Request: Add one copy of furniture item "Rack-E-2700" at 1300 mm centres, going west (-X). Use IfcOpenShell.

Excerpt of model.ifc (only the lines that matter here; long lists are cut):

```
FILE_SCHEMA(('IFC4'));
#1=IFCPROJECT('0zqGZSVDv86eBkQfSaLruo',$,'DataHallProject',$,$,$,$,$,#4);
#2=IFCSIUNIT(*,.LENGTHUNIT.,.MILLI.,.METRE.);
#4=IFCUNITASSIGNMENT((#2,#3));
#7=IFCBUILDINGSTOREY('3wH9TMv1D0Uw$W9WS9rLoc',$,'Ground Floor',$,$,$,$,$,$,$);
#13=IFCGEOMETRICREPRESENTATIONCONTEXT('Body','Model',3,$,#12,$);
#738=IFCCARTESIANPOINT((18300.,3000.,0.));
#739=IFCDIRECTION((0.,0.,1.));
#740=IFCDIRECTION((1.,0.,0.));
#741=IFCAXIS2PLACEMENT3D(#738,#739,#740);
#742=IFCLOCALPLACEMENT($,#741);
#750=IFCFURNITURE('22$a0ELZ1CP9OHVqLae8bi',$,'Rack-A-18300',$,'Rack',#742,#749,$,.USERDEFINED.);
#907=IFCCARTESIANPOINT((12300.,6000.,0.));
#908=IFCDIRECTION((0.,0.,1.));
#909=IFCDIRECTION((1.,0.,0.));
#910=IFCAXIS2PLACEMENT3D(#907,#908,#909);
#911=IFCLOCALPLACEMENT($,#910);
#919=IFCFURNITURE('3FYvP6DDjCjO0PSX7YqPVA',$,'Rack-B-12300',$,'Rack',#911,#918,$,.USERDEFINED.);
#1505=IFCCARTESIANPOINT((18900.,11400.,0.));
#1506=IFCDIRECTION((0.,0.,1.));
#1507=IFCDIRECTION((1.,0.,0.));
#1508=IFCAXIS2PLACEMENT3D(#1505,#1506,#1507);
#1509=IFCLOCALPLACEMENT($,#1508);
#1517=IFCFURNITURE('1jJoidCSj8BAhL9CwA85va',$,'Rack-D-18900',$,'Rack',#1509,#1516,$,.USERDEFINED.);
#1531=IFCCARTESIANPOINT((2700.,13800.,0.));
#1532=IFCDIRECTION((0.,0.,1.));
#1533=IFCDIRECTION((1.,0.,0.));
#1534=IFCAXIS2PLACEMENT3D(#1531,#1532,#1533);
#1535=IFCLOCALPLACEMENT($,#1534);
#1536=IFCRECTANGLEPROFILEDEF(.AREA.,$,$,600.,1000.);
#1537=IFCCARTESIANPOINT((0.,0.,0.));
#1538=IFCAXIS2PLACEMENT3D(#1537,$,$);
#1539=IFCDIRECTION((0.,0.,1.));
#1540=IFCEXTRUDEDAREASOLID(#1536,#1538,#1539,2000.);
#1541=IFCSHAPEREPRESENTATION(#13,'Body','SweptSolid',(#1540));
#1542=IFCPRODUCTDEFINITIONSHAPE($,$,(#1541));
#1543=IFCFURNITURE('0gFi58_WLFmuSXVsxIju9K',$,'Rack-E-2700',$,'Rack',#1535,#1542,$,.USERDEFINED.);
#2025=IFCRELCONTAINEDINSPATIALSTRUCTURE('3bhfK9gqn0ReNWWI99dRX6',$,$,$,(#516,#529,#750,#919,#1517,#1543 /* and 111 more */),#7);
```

```python
import numpy as np
import ifcopenshell
import ifcopenshell.api.geometry
import ifcopenshell.api.root
import ifcopenshell.util.element
import ifcopenshell.util.placement

model = ifcopenshell.open("model.ifc")

source = model.by_guid("0gFi58_WLFmuSXVsxIju9K")
base = ifcopenshell.util.placement.get_local_placement(source.ObjectPlacement)
step = np.array([-1.0, 0.0, 0.0]) * 1300.0

for i in range(1, 2):
    copy = ifcopenshell.api.root.copy_class(model, product=source)
    copy.Representation = ifcopenshell.util.element.copy_deep(
        model, source.Representation, exclude=["IfcGeometricRepresentationContext", "IfcRepresentationMap"]
    )
    matrix = base.copy()
    matrix[:3, 3] += i * step
    print("added at", matrix[:3, 3].round(3) + 0.0)
    ifcopenshell.api.geometry.edit_object_placement(model, product=copy, matrix=matrix, is_si=False)

model.write("model_edited.ifc")
```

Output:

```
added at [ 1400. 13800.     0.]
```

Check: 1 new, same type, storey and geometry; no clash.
